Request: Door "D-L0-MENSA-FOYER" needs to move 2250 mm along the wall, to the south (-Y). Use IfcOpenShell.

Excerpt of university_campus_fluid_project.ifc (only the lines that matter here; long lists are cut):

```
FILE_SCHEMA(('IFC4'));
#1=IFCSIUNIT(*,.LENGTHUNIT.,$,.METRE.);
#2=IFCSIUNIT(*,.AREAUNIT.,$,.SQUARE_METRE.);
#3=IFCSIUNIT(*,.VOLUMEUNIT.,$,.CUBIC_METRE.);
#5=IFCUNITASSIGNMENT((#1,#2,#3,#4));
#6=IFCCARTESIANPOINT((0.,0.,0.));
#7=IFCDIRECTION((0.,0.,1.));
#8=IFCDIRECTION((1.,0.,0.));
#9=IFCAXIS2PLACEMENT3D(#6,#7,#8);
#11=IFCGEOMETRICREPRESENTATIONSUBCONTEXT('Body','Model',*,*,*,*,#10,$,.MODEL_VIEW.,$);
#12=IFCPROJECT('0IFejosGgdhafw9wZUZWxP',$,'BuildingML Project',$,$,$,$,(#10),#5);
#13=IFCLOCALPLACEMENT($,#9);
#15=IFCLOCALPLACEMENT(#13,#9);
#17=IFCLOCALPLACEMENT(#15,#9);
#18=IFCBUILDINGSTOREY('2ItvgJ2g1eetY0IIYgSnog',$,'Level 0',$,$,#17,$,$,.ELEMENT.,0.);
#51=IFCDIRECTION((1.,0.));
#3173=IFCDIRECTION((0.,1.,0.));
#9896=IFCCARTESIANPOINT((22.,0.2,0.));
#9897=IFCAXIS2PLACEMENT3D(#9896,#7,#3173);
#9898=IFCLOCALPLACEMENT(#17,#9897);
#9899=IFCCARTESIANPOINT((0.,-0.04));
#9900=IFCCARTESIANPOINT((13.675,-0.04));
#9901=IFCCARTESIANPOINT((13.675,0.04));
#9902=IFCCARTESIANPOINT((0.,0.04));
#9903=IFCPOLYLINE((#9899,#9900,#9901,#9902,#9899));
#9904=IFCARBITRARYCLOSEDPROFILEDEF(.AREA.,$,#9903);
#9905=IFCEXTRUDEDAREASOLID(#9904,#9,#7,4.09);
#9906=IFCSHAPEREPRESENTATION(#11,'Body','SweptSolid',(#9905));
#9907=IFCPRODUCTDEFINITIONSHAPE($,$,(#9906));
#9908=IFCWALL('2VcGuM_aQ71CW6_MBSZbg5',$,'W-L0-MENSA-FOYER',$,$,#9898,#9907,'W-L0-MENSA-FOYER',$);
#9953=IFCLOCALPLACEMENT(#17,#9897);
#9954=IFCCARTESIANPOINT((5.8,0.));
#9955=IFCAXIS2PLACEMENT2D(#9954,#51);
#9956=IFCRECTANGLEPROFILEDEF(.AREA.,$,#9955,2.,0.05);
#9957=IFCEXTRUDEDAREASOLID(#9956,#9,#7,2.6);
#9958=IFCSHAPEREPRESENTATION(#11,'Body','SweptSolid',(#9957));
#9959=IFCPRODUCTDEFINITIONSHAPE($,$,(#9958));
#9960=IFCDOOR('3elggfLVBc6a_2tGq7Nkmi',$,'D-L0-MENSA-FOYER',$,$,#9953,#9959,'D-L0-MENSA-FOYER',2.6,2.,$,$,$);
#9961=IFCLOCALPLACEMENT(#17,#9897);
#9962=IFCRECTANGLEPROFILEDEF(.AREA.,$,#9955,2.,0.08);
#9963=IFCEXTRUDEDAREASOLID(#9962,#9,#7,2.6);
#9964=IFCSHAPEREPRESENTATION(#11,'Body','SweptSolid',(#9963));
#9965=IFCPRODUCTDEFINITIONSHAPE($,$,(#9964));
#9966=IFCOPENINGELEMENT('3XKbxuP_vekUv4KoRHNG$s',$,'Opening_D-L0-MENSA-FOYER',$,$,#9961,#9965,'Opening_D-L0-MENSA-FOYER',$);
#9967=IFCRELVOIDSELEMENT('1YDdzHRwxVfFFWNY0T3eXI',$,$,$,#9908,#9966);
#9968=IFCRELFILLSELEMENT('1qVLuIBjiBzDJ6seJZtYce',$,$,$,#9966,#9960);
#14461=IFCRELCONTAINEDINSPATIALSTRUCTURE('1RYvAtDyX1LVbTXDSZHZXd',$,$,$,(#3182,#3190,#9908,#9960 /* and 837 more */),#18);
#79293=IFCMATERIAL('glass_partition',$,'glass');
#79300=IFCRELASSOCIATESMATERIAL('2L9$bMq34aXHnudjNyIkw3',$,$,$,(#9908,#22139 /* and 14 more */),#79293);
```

```python
import ifcopenshell
import ifcopenshell.api.geometry
import ifcopenshell.util.placement
import ifcopenshell.util.unit

model = ifcopenshell.open("university_campus_fluid_project.ifc")
unit_scale = ifcopenshell.util.unit.calculate_unit_scale(model)

door = model.by_guid("3elggfLVBc6a_2tGq7Nkmi")
opening = door.FillsVoids[0].RelatingOpeningElement
wall = opening.VoidsElements[0].RelatingBuildingElement

wall_matrix = ifcopenshell.util.placement.get_local_placement(wall.ObjectPlacement)
shift = wall_matrix[:3, 0] * -2.25 / unit_scale
before = ifcopenshell.util.placement.get_local_placement(door.ObjectPlacement)[:3, 3].copy()

# The door is not placed relative to its opening, so move both.
for product in (opening, door):
    matrix = ifcopenshell.util.placement.get_local_placement(product.ObjectPlacement)
    matrix[:3, 3] += shift
    ifcopenshell.api.geometry.edit_object_placement(model, product=product, matrix=matrix, is_si=False)

after = ifcopenshell.util.placement.get_local_placement(door.ObjectPlacement)[:3, 3]
print("door moved by", (after - before).round(3) + 0.0)

model.write("university_campus_fluid_project_edited.ifc")
```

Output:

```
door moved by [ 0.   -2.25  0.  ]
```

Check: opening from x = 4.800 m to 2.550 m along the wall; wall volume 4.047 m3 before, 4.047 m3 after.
